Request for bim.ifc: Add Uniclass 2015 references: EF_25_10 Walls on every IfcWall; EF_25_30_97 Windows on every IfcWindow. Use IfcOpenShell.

First a look at what the model holds.

```python
import ifcopenshell

model = ifcopenshell.open("bim.ifc")
print(model.schema)
print("classifications:", [c.Name for c in model.by_type("IfcClassification")])
for ifc_class in ("IfcDoor", "IfcRoof", "IfcStair", "IfcWall", "IfcWindow"):
    print(ifc_class, len(model.by_type(ifc_class)))
```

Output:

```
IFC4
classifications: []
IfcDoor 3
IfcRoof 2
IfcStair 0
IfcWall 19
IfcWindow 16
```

```python
import ifcopenshell
import ifcopenshell.api.classification

model = ifcopenshell.open("bim.ifc")

system = ifcopenshell.api.classification.add_classification(model, classification="Uniclass 2015")

codes = {
    "IfcWall": ("EF_25_10", "Walls"),
    "IfcWindow": ("EF_25_30_97", "Windows"),
}
for ifc_class, (code, name) in codes.items():
    products = model.by_type(ifc_class)
    ifcopenshell.api.classification.add_reference(
        model, products=products, classification=system, identification=code, name=name
    )
    print(code, len(products))

model.write("bim_updated.ifc")
```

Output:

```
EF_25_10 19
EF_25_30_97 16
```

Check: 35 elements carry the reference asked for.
